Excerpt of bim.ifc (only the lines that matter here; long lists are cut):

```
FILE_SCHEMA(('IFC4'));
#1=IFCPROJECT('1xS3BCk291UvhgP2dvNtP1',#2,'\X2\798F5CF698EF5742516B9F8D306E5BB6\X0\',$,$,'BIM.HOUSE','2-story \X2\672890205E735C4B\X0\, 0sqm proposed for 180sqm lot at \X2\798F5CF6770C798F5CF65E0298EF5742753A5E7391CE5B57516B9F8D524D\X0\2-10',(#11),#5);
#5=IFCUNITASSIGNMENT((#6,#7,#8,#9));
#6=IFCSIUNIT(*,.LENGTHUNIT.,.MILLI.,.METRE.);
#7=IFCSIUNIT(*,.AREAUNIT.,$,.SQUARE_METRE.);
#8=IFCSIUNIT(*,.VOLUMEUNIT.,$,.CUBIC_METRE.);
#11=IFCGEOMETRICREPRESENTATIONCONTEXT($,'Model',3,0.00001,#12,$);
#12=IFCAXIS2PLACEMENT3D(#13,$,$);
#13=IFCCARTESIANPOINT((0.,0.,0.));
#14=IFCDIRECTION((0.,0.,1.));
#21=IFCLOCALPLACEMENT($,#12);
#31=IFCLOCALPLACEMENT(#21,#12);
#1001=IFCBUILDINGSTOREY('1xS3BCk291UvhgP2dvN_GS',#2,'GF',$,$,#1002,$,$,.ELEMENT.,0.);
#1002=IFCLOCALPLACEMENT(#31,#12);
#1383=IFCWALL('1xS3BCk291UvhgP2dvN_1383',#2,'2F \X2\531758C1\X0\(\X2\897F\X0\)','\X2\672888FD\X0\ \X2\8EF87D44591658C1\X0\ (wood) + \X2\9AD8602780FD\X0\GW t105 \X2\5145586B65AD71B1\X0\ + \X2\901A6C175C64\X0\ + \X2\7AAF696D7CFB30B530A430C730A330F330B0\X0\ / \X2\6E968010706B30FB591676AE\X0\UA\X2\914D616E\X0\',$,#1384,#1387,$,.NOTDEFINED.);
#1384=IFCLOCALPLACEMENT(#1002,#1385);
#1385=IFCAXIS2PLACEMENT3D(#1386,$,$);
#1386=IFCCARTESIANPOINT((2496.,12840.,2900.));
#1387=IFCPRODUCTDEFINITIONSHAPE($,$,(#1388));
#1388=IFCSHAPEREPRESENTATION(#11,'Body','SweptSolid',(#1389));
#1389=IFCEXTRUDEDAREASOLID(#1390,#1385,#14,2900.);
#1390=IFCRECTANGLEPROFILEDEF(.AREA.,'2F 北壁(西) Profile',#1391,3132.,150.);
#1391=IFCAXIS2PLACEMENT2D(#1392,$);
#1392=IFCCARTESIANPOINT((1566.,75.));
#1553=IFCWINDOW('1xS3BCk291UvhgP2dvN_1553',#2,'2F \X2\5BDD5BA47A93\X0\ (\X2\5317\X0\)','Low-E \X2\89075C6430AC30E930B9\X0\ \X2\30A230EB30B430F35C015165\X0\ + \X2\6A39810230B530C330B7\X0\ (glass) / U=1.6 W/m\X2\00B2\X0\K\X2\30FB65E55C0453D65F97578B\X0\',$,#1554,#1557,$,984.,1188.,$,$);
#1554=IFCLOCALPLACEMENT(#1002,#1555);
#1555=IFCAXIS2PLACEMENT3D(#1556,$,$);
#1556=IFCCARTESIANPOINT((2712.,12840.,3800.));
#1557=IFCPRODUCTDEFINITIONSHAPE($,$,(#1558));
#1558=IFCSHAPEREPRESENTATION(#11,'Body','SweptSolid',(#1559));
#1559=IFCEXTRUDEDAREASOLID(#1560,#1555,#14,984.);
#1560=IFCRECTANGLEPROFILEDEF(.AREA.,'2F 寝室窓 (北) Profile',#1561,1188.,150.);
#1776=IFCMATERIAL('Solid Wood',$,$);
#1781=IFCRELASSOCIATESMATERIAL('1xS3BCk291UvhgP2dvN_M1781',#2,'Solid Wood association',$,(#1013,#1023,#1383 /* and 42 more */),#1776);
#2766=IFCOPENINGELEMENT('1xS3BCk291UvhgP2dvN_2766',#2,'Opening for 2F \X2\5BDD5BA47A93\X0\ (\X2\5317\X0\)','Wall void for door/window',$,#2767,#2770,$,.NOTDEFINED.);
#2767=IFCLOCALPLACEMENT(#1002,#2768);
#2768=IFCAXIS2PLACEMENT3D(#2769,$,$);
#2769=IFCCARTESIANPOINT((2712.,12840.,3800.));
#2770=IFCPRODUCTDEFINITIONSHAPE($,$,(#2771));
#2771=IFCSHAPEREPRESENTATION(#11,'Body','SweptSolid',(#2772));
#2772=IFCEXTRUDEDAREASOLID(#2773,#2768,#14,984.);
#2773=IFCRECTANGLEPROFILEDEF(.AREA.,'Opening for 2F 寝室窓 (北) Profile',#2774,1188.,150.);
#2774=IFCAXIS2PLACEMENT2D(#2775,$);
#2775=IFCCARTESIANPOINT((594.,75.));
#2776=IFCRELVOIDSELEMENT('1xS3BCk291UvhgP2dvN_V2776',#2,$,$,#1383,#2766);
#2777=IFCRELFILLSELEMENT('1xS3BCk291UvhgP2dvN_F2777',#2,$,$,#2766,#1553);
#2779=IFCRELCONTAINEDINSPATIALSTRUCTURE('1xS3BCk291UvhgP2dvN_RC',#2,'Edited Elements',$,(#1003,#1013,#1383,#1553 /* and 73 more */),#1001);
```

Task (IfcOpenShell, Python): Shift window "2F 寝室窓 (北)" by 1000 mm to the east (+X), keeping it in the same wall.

```python
import ifcopenshell
import ifcopenshell.api.geometry
import ifcopenshell.util.placement
import ifcopenshell.util.unit

model = ifcopenshell.open("bim.ifc")
unit_scale = ifcopenshell.util.unit.calculate_unit_scale(model)

window = model.by_id(1553)
opening = window.FillsVoids[0].RelatingOpeningElement
wall = opening.VoidsElements[0].RelatingBuildingElement

wall_matrix = ifcopenshell.util.placement.get_local_placement(wall.ObjectPlacement)
shift = wall_matrix[:3, 0] * 1 / unit_scale
before = ifcopenshell.util.placement.get_local_placement(window.ObjectPlacement)[:3, 3].copy()

# The window is not placed relative to its opening, so move both.
for product in (opening, window):
    matrix = ifcopenshell.util.placement.get_local_placement(product.ObjectPlacement)
    matrix[:3, 3] += shift
    ifcopenshell.api.geometry.edit_object_placement(model, product=product, matrix=matrix, is_si=False)

after = ifcopenshell.util.placement.get_local_placement(window.ObjectPlacement)[:3, 3]
print("window moved by", (after - before).round(3) + 0.0)

model.write("bim-out.ifc")
```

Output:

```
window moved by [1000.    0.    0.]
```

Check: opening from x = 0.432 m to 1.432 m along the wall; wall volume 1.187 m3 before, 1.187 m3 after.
